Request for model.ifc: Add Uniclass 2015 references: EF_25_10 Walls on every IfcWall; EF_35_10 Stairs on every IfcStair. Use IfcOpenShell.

First a look at what the model holds.

```python
import ifcopenshell

model = ifcopenshell.open("model.ifc")
print(model.schema)
print("classifications:", [c.Name for c in model.by_type("IfcClassification")])
for ifc_class in ("IfcDoor", "IfcRoof", "IfcStair", "IfcWall", "IfcWindow"):
    print(ifc_class, len(model.by_type(ifc_class)))
```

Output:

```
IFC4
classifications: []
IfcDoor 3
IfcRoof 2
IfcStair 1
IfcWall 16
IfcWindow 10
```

```python
import ifcopenshell
import ifcopenshell.api.classification

model = ifcopenshell.open("model.ifc")

system = ifcopenshell.api.classification.add_classification(model, classification="Uniclass 2015")

codes = {
    "IfcWall": ("EF_25_10", "Walls"),
    "IfcStair": ("EF_35_10", "Stairs"),
}
for ifc_class, (code, name) in codes.items():
    products = model.by_type(ifc_class)
    ifcopenshell.api.classification.add_reference(
        model, products=products, classification=system, identification=code, name=name
    )
    print(code, len(products))

model.write("model-out.ifc")
```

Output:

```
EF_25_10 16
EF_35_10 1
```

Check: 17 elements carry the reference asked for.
